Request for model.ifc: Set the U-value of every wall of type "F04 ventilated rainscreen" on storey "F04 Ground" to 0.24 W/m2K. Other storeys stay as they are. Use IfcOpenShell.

First a look at what the model holds.

```python
import ifcopenshell
import ifcopenshell.util.element

model = ifcopenshell.open("model.ifc")
print(model.schema)
storey = next(s for s in model.by_type("IfcBuildingStorey") if s.Name == "F04 Ground")
walls = [e for e in ifcopenshell.util.element.get_decomposition(storey) if e.is_a("IfcWall")]
seen = {}
for e in walls:
    element_type = ifcopenshell.util.element.get_type(e)
    key = (element_type.Name if element_type != e and element_type else None, ifcopenshell.util.element.get_pset(e, "Pset_WallCommon", "ThermalTransmittance"))
    seen[key] = seen.get(key, 0) + 1
for (name, value), count in sorted(seen.items(), key=str):
    print(count, "x", name, "|", value)
```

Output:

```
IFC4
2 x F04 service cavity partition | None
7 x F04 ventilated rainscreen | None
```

```python
import ifcopenshell
import ifcopenshell.api.pset
import ifcopenshell.util.element

model = ifcopenshell.open("model.ifc")

storey = next(s for s in model.by_type("IfcBuildingStorey") if s.Name == "F04 Ground")
walls = [e for e in ifcopenshell.util.element.get_decomposition(storey) if e.is_a("IfcWall")]

count = 0
for e in walls:
    element_type = ifcopenshell.util.element.get_type(e)
    if element_type in (None, e) or element_type.Name != "F04 ventilated rainscreen":
        continue
    # add_pset returns the element's existing set when there is one.
    pset = ifcopenshell.api.pset.add_pset(model, product=e, name="Pset_WallCommon")
    ifcopenshell.api.pset.edit_pset(model, pset=pset, properties={"ThermalTransmittance": 0.24})
    count += 1

print(count, "walls updated")

model.write("model-out.ifc")
```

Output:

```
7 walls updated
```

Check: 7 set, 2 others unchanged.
